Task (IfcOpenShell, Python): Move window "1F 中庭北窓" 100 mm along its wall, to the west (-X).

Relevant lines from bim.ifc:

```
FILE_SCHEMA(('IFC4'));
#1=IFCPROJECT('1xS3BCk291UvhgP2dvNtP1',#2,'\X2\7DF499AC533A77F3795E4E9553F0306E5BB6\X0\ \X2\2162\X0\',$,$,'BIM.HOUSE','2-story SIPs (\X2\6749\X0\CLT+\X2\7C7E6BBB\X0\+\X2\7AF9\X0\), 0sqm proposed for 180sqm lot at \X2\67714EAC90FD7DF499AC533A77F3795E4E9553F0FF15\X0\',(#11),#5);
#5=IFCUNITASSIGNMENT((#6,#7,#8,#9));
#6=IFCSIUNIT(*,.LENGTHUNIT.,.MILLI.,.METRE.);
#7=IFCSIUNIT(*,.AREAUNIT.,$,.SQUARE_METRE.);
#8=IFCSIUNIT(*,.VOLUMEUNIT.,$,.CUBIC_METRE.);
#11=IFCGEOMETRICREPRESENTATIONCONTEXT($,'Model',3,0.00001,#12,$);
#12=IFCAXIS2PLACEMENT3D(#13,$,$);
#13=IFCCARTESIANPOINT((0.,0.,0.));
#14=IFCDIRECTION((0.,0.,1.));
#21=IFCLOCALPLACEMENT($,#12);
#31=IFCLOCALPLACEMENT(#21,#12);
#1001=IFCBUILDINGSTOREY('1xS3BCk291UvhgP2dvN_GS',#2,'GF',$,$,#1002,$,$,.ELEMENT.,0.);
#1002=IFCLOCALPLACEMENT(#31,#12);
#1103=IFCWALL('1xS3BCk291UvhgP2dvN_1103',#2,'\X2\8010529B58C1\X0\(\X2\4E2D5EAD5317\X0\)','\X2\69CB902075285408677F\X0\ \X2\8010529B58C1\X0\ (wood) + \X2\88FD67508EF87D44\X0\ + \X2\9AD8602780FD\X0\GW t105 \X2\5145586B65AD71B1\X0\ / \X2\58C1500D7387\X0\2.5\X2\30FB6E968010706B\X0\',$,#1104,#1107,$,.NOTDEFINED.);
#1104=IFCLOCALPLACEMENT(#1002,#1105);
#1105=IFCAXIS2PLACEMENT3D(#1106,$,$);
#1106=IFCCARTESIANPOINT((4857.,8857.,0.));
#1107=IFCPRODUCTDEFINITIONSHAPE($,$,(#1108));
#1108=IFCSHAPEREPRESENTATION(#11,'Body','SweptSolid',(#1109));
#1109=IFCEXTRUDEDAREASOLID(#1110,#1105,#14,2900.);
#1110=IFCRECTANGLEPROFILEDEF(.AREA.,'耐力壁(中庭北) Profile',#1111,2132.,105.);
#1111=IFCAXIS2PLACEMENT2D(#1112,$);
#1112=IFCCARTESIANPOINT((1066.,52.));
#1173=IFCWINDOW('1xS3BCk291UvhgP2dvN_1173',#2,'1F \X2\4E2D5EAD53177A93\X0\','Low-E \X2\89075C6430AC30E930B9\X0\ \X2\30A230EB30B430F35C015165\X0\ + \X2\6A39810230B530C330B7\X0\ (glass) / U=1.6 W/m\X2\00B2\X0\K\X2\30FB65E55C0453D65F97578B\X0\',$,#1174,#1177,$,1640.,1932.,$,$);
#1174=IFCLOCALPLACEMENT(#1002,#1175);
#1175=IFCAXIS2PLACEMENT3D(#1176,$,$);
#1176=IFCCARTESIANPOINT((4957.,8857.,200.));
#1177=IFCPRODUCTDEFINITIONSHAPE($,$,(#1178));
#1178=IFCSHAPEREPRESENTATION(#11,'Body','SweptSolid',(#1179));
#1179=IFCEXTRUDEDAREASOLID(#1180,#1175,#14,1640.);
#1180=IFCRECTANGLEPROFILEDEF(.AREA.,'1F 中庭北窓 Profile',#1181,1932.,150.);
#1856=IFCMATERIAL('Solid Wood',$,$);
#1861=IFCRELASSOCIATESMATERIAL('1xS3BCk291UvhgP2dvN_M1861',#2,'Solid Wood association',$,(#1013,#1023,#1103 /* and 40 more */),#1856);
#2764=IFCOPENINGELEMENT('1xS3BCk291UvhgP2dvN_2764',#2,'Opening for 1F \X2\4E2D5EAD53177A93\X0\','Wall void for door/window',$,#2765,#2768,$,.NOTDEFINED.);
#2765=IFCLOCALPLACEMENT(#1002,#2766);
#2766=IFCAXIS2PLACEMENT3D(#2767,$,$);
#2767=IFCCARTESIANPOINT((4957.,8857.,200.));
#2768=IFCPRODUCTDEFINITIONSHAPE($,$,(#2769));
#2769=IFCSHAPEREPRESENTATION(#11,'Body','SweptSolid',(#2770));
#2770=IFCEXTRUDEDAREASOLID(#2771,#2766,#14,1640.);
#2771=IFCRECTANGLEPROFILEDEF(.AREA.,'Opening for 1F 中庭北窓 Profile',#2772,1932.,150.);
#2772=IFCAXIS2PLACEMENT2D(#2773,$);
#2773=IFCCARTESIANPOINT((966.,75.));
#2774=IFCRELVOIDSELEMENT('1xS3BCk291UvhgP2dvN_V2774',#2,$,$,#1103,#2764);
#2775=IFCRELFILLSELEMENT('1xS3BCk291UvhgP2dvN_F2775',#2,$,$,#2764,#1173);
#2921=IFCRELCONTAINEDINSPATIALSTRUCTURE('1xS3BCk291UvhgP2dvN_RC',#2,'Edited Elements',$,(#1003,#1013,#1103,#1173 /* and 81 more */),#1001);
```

```python
import ifcopenshell
import ifcopenshell.api.geometry
import ifcopenshell.util.placement
import ifcopenshell.util.unit

model = ifcopenshell.open("bim.ifc")
unit_scale = ifcopenshell.util.unit.calculate_unit_scale(model)

window = model.by_guid("1xS3BCk291UvhgP2dvN_1173")
opening = window.FillsVoids[0].RelatingOpeningElement
wall = opening.VoidsElements[0].RelatingBuildingElement

wall_matrix = ifcopenshell.util.placement.get_local_placement(wall.ObjectPlacement)
shift = wall_matrix[:3, 0] * -0.1 / unit_scale
before = ifcopenshell.util.placement.get_local_placement(window.ObjectPlacement)[:3, 3].copy()

# The window is not placed relative to its opening, so move both.
for product in (opening, window):
    matrix = ifcopenshell.util.placement.get_local_placement(product.ObjectPlacement)
    matrix[:3, 3] += shift
    ifcopenshell.api.geometry.edit_object_placement(model, product=product, matrix=matrix, is_si=False)

after = ifcopenshell.util.placement.get_local_placement(window.ObjectPlacement)[:3, 3]
print("window moved by", (after - before).round(3) + 0.0)

model.write("bim_rev.ifc")
```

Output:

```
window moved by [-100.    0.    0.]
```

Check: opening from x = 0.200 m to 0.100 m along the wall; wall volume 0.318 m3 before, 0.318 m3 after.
